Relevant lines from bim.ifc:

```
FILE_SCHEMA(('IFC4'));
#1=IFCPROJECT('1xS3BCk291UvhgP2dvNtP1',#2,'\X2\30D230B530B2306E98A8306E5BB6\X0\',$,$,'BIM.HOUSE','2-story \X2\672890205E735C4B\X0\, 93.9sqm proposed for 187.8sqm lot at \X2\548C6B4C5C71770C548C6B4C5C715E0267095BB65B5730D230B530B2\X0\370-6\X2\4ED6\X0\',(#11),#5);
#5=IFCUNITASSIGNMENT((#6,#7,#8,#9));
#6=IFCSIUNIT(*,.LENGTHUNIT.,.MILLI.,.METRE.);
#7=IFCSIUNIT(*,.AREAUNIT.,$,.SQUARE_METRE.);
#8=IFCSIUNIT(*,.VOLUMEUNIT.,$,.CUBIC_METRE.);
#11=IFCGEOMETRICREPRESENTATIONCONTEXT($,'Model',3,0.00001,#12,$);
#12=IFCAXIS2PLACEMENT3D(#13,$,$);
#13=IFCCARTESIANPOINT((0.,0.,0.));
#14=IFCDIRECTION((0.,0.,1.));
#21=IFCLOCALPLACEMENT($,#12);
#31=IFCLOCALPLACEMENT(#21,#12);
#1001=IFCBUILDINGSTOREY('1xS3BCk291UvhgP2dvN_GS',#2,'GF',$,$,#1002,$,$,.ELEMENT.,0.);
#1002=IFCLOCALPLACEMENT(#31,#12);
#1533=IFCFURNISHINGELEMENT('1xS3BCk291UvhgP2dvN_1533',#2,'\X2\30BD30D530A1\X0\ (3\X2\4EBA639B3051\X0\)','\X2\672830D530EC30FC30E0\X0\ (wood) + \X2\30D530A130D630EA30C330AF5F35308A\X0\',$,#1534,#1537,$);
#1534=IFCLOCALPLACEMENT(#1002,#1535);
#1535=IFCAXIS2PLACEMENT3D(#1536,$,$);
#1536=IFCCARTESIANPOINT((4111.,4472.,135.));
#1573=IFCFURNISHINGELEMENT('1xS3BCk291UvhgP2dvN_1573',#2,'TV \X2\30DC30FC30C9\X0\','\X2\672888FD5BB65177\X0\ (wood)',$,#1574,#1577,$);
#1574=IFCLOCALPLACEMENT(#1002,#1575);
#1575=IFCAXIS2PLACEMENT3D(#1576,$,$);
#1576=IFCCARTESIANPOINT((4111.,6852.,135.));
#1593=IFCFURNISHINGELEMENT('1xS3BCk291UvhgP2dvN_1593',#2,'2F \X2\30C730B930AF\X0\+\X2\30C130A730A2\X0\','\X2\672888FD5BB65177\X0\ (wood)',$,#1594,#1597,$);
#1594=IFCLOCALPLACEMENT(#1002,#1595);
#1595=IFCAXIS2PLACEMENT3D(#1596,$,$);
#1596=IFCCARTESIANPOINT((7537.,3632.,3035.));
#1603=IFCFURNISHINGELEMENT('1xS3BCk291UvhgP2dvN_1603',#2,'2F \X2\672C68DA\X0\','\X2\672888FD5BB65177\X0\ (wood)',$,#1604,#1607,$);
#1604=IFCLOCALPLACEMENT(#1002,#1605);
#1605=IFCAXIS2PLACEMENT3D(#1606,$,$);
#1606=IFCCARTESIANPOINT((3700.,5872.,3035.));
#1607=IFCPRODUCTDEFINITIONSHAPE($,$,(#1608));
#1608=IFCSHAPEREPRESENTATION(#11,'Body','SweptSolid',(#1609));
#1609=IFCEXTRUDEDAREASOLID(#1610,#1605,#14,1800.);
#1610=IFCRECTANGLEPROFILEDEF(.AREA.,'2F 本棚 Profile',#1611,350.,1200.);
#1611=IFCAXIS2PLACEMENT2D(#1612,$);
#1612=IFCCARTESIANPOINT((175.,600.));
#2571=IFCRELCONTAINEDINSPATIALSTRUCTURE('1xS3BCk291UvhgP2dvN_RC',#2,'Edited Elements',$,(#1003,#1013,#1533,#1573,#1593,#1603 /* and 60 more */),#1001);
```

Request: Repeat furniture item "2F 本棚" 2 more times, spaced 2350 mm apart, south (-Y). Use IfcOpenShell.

```python
import numpy as np
import ifcopenshell
import ifcopenshell.api.geometry
import ifcopenshell.api.root
import ifcopenshell.util.element
import ifcopenshell.util.placement
import ifcopenshell.util.unit

model = ifcopenshell.open("bim.ifc")
unit_scale = ifcopenshell.util.unit.calculate_unit_scale(model)


def reuse_history(source, copy):
    """copy_class also copies each property set's owner history, people and application; keep the originals."""
    for rel in copy.IsDefinedBy:
        if rel.is_a("IfcRelDefinesByProperties") and (history := rel.RelatingPropertyDefinition.OwnerHistory):
            rel.RelatingPropertyDefinition.OwnerHistory = source.OwnerHistory
            ifcopenshell.util.element.remove_deep2(model, history)


source = model.by_guid("1xS3BCk291UvhgP2dvN_1603")
base = ifcopenshell.util.placement.get_local_placement(source.ObjectPlacement)
step = np.array([0.0, -1.0, 0.0]) * 2.35 / unit_scale

for i in range(1, 3):
    copy = ifcopenshell.api.root.copy_class(model, product=source)
    copy.Representation = ifcopenshell.util.element.copy_deep(
        model, source.Representation, exclude=["IfcGeometricRepresentationContext", "IfcRepresentationMap"]
    )
    reuse_history(source, copy)
    matrix = base.copy()
    matrix[:3, 3] += i * step
    print("added at", matrix[:3, 3].round(3) + 0.0)
    ifcopenshell.api.geometry.edit_object_placement(model, product=copy, matrix=matrix, is_si=False)

model.write("bim_rev.ifc")
```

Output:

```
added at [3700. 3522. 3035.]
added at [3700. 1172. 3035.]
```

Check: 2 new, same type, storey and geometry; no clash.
